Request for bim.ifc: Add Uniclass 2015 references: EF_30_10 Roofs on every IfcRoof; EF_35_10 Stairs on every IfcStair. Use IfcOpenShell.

First a look at what the model holds.

```python
import ifcopenshell

model = ifcopenshell.open("bim.ifc")
print(model.schema)
print("classifications:", [c.Name for c in model.by_type("IfcClassification")])
for ifc_class in ("IfcDoor", "IfcRoof", "IfcStair", "IfcWall", "IfcWindow"):
    print(ifc_class, len(model.by_type(ifc_class)))
```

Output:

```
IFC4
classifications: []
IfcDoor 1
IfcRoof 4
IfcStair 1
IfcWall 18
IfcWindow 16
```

```python
import ifcopenshell
import ifcopenshell.api.classification

model = ifcopenshell.open("bim.ifc")

system = ifcopenshell.api.classification.add_classification(model, classification="Uniclass 2015")

codes = {
    "IfcRoof": ("EF_30_10", "Roofs"),
    "IfcStair": ("EF_35_10", "Stairs"),
}
for ifc_class, (code, name) in codes.items():
    products = model.by_type(ifc_class)
    ifcopenshell.api.classification.add_reference(
        model, products=products, classification=system, identification=code, name=name
    )
    print(code, len(products))

model.write("bim_edited.ifc")
```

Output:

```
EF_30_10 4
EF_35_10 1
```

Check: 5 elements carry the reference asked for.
